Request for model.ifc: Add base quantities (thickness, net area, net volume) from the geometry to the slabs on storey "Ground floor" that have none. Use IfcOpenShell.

First a look at what the model holds.

```python
import ifcopenshell
import ifcopenshell.util.element
import ifcopenshell.util.unit

model = ifcopenshell.open("model.ifc")
print(model.schema)
for unit_type in ("LENGTHUNIT", "AREAUNIT", "VOLUMEUNIT"):
    print(unit_type, ifcopenshell.util.unit.calculate_unit_scale(model, unit_type))
storey = next(s for s in model.by_type("IfcBuildingStorey") if s.Name == "Ground floor")
slabs = [e for e in ifcopenshell.util.element.get_decomposition(storey) if e.is_a("IfcSlab")]
for e in sorted(slabs, key=lambda e: e.id()):
    print(e.id(), e.is_a(), e.Name, list(ifcopenshell.util.element.get_psets(e, qtos_only=True)), sep=" | ")
```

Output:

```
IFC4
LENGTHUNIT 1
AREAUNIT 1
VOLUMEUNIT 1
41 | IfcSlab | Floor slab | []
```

```python
import ifcopenshell
import ifcopenshell.api.pset
import ifcopenshell.geom
import ifcopenshell.util.element
import ifcopenshell.util.shape
import ifcopenshell.util.unit

model = ifcopenshell.open("model.ifc")
unit_scale = ifcopenshell.util.unit.calculate_unit_scale(model)
area_scale = ifcopenshell.util.unit.calculate_unit_scale(model, "AREAUNIT")
volume_scale = ifcopenshell.util.unit.calculate_unit_scale(model, "VOLUMEUNIT")
settings = ifcopenshell.geom.settings()

storey = next(s for s in model.by_type("IfcBuildingStorey") if s.Name == "Ground floor")
slabs = [e for e in ifcopenshell.util.element.get_decomposition(storey) if e.is_a("IfcSlab")]

for e in sorted(slabs, key=lambda e: e.id()):
    if ifcopenshell.util.element.get_psets(e, qtos_only=True, should_inherit=False):
        continue
    # Geometry comes back in metres, in the element's own axes.
    shape = ifcopenshell.geom.create_shape(settings, e)
    values = {
        "Width": ifcopenshell.util.shape.get_z(shape.geometry) / unit_scale,
        "NetArea": ifcopenshell.util.shape.get_footprint_area(shape.geometry) / area_scale,
        "NetVolume": ifcopenshell.util.shape.get_volume(shape.geometry) / volume_scale,
    }
    qto = ifcopenshell.api.pset.add_qto(model, product=e, name="Qto_SlabBaseQuantities")
    ifcopenshell.api.pset.edit_qto(model, qto=qto, properties=values)
    print(e.id(), {k: round(v, 3) for k, v in values.items()})

model.write("model_updated.ifc")
```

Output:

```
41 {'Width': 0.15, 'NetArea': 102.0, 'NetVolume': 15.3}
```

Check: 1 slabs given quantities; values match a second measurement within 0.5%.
